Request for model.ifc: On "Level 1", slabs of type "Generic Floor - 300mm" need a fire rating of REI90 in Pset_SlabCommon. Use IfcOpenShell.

First a look at what the model holds.

```python
import ifcopenshell
import ifcopenshell.util.element

model = ifcopenshell.open("model.ifc")
print(model.schema)
storey = next(s for s in model.by_type("IfcBuildingStorey") if s.Name == "Level 1")
slabs = [e for e in ifcopenshell.util.element.get_decomposition(storey) if e.is_a("IfcSlab")]
seen = {}
for e in slabs:
    element_type = ifcopenshell.util.element.get_type(e)
    key = (element_type.Name if element_type != e and element_type else None, ifcopenshell.util.element.get_pset(e, "Pset_SlabCommon", "FireRating"))
    seen[key] = seen.get(key, 0) + 1
for (name, value), count in sorted(seen.items(), key=str):
    print(count, "x", name, "|", value)
```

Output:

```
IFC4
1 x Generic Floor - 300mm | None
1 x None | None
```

```python
import ifcopenshell
import ifcopenshell.api.pset
import ifcopenshell.util.element

model = ifcopenshell.open("model.ifc")

storey = next(s for s in model.by_type("IfcBuildingStorey") if s.Name == "Level 1")
slabs = [e for e in ifcopenshell.util.element.get_decomposition(storey) if e.is_a("IfcSlab")]

count = 0
for e in slabs:
    element_type = ifcopenshell.util.element.get_type(e)
    if element_type in (None, e) or element_type.Name != "Generic Floor - 300mm":
        continue
    # add_pset returns the element's existing set when there is one.
    pset = ifcopenshell.api.pset.add_pset(model, product=e, name="Pset_SlabCommon")
    ifcopenshell.api.pset.edit_pset(model, pset=pset, properties={"FireRating": "REI90"})
    count += 1

print(count, "slabs updated")

model.write("model_updated.ifc")
```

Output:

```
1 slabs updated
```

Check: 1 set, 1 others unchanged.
